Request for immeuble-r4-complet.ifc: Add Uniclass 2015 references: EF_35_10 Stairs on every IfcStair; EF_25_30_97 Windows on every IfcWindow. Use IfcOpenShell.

First a look at what the model holds.

```python
import ifcopenshell

model = ifcopenshell.open("immeuble-r4-complet.ifc")
print(model.schema)
print("classifications:", [c.Name for c in model.by_type("IfcClassification")])
for ifc_class in ("IfcDoor", "IfcRoof", "IfcStair", "IfcWall", "IfcWindow"):
    print(ifc_class, len(model.by_type(ifc_class)))
```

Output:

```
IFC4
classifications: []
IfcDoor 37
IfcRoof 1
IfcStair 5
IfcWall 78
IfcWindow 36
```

```python
import ifcopenshell
import ifcopenshell.api.classification

model = ifcopenshell.open("immeuble-r4-complet.ifc")

system = ifcopenshell.api.classification.add_classification(model, classification="Uniclass 2015")

codes = {
    "IfcStair": ("EF_35_10", "Stairs"),
    "IfcWindow": ("EF_25_30_97", "Windows"),
}
for ifc_class, (code, name) in codes.items():
    products = model.by_type(ifc_class)
    ifcopenshell.api.classification.add_reference(
        model, products=products, classification=system, identification=code, name=name
    )
    print(code, len(products))

model.write("immeuble-r4-complet_rev.ifc")
```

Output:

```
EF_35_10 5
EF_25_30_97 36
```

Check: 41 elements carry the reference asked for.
